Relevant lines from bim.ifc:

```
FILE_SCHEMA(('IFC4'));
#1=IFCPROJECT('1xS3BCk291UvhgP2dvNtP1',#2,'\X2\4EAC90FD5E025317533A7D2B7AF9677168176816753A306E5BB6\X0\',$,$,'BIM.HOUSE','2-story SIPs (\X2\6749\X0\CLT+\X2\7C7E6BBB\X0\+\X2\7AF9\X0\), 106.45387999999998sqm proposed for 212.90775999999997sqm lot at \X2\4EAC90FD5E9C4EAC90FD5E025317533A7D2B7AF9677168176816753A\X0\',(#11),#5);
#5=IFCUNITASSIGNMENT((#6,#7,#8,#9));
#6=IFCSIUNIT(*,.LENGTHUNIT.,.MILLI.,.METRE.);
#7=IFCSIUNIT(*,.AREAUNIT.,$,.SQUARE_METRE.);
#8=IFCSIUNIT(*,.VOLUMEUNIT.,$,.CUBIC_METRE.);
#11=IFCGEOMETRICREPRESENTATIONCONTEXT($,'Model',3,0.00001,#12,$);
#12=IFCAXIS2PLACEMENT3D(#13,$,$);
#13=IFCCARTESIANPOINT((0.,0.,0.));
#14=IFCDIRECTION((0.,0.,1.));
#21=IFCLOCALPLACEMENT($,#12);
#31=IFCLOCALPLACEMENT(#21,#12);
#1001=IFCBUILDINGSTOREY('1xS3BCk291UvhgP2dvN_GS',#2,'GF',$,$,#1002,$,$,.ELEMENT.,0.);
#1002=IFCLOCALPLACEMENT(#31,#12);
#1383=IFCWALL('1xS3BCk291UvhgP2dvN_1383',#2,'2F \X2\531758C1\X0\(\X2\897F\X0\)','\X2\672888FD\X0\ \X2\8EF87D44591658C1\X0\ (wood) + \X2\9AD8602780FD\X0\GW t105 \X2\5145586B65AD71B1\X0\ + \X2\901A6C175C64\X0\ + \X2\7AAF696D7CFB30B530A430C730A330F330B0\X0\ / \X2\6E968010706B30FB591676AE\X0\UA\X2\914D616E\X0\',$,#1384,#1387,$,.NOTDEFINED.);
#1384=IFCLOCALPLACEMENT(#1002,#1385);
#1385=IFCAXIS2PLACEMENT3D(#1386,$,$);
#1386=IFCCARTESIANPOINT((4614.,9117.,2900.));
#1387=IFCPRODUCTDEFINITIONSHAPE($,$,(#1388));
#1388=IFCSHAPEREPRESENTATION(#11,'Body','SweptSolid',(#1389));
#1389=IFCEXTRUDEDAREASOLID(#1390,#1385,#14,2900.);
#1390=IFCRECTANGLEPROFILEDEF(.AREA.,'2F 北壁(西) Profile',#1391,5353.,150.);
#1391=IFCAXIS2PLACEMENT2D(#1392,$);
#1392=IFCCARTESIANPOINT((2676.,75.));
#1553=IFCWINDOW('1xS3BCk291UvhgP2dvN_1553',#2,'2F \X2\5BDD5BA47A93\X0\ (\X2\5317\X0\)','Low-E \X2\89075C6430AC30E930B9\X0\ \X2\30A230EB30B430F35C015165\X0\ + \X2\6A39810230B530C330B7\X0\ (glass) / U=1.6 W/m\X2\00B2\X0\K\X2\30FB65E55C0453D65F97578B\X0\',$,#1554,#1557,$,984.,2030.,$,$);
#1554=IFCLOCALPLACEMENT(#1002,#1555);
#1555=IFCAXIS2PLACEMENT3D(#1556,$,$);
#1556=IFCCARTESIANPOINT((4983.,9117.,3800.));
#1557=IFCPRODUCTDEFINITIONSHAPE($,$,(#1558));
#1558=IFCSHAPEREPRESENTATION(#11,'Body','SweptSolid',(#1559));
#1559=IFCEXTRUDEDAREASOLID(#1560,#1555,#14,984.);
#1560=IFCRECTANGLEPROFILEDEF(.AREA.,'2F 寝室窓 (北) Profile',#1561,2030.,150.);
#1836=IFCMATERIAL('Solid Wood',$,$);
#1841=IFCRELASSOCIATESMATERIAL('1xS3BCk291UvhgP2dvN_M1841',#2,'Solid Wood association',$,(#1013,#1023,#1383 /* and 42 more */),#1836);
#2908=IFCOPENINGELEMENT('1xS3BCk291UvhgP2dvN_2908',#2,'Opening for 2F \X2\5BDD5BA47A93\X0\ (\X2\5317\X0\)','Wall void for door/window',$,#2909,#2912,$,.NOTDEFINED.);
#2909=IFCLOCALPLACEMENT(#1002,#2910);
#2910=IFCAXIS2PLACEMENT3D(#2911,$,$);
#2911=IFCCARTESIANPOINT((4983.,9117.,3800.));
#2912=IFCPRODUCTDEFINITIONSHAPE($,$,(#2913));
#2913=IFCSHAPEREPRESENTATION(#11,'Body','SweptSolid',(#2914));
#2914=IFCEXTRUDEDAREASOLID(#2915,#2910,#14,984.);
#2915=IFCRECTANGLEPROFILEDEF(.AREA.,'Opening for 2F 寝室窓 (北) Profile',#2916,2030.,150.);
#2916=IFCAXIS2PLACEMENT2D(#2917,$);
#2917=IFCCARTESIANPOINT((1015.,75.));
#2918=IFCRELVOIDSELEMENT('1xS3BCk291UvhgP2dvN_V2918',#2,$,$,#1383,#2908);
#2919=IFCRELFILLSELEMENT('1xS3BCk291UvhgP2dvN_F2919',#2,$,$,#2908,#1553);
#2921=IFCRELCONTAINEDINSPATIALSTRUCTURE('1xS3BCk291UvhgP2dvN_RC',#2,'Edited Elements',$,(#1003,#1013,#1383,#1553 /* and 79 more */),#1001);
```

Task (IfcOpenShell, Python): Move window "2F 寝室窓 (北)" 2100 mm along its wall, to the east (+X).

```python
import ifcopenshell
import ifcopenshell.api.geometry
import ifcopenshell.util.placement

model = ifcopenshell.open("bim.ifc")

window = model.by_guid("1xS3BCk291UvhgP2dvN_1553")
opening = window.FillsVoids[0].RelatingOpeningElement
wall = opening.VoidsElements[0].RelatingBuildingElement

wall_matrix = ifcopenshell.util.placement.get_local_placement(wall.ObjectPlacement)
shift = wall_matrix[:3, 0] * 2100.0
before = ifcopenshell.util.placement.get_local_placement(window.ObjectPlacement)[:3, 3].copy()

# The window is not placed relative to its opening, so move both.
for product in (opening, window):
    matrix = ifcopenshell.util.placement.get_local_placement(product.ObjectPlacement)
    matrix[:3, 3] += shift
    ifcopenshell.api.geometry.edit_object_placement(model, product=product, matrix=matrix, is_si=False)

after = ifcopenshell.util.placement.get_local_placement(window.ObjectPlacement)[:3, 3]
print("window moved by", (after - before).round(3) + 0.0)

model.write("bim_v2.ifc")
```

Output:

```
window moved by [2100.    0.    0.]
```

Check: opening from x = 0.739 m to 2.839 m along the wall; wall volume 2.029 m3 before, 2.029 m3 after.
